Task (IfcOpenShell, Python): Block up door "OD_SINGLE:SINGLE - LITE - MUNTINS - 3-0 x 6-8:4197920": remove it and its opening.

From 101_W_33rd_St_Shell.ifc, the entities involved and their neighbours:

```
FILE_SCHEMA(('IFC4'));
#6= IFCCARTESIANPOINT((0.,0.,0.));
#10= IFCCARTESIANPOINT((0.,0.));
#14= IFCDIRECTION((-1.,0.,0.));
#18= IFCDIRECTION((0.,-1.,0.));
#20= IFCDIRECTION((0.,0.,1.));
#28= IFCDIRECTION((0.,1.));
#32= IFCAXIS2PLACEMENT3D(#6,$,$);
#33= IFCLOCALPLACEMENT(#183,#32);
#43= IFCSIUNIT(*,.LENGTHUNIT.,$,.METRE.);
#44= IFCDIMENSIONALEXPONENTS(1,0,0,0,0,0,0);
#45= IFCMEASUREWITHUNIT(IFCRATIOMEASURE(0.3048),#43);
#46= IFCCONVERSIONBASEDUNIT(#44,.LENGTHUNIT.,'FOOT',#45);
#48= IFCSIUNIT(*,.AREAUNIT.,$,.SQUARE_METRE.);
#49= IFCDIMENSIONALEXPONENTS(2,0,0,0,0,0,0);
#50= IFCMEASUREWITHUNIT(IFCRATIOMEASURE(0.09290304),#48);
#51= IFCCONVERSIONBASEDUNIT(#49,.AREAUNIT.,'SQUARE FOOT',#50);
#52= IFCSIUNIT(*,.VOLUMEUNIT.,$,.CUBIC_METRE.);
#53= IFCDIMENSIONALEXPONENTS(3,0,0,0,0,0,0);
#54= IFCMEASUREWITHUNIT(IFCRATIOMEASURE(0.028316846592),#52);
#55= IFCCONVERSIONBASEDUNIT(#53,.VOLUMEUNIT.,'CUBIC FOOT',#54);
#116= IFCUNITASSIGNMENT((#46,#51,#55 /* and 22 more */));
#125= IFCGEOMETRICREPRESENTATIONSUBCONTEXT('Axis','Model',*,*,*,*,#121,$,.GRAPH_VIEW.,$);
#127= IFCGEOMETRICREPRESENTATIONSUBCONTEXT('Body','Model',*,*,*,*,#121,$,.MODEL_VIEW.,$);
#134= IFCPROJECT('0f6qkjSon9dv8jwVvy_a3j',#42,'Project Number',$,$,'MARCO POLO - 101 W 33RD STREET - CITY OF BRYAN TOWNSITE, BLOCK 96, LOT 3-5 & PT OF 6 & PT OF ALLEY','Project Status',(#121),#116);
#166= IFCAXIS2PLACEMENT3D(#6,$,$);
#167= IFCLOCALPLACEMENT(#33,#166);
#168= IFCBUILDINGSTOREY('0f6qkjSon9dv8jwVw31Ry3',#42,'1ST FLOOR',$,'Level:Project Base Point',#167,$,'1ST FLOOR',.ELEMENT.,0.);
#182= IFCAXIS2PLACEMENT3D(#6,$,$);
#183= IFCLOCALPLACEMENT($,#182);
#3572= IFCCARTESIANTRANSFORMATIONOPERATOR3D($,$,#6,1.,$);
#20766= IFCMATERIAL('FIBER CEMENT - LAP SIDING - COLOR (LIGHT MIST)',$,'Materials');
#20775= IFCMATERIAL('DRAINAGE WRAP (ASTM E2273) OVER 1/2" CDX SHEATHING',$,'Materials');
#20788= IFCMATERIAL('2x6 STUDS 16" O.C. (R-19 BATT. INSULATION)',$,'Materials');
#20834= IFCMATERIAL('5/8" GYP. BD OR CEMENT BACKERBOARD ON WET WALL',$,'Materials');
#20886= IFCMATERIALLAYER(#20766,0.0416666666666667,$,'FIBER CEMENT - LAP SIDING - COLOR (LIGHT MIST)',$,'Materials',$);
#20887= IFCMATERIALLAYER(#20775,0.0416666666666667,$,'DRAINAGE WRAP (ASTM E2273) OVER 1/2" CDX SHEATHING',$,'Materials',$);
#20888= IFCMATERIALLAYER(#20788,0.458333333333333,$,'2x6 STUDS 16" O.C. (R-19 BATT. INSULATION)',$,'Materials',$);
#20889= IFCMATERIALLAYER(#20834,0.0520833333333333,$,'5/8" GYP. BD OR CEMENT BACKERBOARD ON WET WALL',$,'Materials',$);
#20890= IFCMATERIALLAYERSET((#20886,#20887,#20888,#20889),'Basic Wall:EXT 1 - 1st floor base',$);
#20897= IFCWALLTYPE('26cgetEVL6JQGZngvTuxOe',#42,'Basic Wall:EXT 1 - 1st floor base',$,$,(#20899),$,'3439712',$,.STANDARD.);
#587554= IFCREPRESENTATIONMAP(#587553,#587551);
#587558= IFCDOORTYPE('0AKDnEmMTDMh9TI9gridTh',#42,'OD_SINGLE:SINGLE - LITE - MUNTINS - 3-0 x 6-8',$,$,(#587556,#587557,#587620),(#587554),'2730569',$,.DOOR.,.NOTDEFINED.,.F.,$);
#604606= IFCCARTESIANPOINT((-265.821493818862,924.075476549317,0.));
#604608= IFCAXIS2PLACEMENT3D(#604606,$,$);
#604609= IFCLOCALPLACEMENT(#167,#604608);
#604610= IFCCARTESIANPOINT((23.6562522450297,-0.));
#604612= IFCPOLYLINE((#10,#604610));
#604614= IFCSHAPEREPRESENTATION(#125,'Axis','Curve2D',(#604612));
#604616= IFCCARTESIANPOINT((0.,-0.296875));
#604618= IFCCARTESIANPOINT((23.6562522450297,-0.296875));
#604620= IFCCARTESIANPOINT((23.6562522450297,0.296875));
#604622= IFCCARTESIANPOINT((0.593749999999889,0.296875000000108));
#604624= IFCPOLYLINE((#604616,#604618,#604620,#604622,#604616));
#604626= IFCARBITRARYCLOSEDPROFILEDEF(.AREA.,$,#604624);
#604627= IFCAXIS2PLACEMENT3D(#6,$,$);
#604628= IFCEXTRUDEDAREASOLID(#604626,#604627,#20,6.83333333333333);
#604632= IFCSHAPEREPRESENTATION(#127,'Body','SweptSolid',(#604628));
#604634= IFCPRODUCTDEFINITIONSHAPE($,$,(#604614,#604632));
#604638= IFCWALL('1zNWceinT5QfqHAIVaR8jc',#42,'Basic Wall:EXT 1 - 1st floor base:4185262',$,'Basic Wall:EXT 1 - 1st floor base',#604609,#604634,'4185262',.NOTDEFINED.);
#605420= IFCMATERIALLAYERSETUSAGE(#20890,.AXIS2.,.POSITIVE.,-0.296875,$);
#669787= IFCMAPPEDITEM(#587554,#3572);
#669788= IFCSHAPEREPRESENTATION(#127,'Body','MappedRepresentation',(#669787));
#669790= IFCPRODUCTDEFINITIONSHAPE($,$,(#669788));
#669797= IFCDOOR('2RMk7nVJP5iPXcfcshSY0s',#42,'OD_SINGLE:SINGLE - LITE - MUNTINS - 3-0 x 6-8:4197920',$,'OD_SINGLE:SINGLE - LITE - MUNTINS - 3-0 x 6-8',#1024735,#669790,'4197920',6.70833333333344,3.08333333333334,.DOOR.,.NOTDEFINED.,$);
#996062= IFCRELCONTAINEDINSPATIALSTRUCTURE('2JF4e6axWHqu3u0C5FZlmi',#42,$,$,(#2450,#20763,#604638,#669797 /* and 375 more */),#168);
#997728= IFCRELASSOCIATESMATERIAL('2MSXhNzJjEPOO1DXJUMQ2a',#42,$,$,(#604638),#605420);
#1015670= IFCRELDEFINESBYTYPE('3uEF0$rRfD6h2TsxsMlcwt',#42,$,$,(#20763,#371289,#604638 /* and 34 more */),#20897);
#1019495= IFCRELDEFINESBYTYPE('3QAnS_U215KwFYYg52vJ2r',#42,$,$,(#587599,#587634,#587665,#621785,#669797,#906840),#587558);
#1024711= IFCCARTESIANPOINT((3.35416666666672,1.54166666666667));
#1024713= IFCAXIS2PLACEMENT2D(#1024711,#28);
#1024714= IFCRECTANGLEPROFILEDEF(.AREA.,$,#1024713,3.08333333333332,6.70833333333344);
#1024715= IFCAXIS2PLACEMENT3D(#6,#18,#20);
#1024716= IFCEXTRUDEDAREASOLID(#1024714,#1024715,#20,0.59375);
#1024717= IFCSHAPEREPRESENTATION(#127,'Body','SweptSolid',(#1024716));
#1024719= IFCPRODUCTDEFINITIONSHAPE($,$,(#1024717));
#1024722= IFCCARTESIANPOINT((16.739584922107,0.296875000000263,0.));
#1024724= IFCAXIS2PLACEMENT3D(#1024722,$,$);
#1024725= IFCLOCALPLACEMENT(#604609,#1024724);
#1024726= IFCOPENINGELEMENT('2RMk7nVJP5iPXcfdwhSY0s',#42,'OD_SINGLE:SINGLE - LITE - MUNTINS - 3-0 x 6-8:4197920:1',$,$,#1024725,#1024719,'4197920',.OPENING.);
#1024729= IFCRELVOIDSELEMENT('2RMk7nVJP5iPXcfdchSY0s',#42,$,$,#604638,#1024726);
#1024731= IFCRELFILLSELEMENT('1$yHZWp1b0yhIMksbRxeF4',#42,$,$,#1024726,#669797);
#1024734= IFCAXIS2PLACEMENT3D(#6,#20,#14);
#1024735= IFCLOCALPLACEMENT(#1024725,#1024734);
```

```python
import ifcopenshell
import ifcopenshell.api.feature
import ifcopenshell.api.root
import ifcopenshell.geom
import ifcopenshell.util.shape

model = ifcopenshell.open("101_W_33rd_St_Shell.ifc")
settings = ifcopenshell.geom.settings()


def volume(element):
    """Net volume in cubic metres, openings subtracted."""
    shape = ifcopenshell.geom.create_shape(settings, element)
    return ifcopenshell.util.shape.get_volume(shape.geometry)


door = model.by_id(669797)
opening = door.FillsVoids[0].RelatingOpeningElement
wall = opening.VoidsElements[0].RelatingBuildingElement
before = volume(wall)

ifcopenshell.api.root.remove_product(model, product=door)
ifcopenshell.api.feature.remove_feature(model, feature=opening)

after = volume(wall)

print(f"wall volume {before:.3f} -> {after:.3f} m3")

model.write("101_W_33rd_St_Shell_v2.ifc")
```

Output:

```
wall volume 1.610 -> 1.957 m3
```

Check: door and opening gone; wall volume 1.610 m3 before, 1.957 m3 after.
